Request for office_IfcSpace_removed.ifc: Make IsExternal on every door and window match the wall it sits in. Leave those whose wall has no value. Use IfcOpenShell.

First a look at what the model holds.

```python
import ifcopenshell
import ifcopenshell.util.element

model = ifcopenshell.open("office_IfcSpace_removed.ifc")
print(model.schema)
seen = {}
for e in model.by_type("IfcDoor") + model.by_type("IfcWindow"):
    if not e.FillsVoids:
        continue
    host = e.FillsVoids[0].RelatingOpeningElement.VoidsElements[0].RelatingBuildingElement
    own = ifcopenshell.util.element.get_pset(e, f"Pset_{e.is_a()[3:].removesuffix('StandardCase')}Common", "IsExternal")
    wall = ifcopenshell.util.element.get_pset(host, "Pset_WallCommon", "IsExternal")
    seen[e.is_a(), own, wall] = seen.get((e.is_a(), own, wall), 0) + 1
for (cls, own, wall), count in sorted(seen.items(), key=str):
    print(count, cls, "IsExternal:", own, "| host wall:", wall)
```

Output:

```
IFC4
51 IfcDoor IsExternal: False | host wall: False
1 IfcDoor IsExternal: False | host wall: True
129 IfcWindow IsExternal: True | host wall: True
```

```python
import ifcopenshell
import ifcopenshell.api.pset
import ifcopenshell.util.element

model = ifcopenshell.open("office_IfcSpace_removed.ifc")

count = 0
for ifc_class, pset_name in (("IfcDoor", "Pset_DoorCommon"), ("IfcWindow", "Pset_WindowCommon")):
    for e in model.by_type(ifc_class):
        if not e.FillsVoids:
            continue
        host = e.FillsVoids[0].RelatingOpeningElement.VoidsElements[0].RelatingBuildingElement
        external = ifcopenshell.util.element.get_pset(host, "Pset_WallCommon", "IsExternal")
        if external is None or ifcopenshell.util.element.get_pset(e, pset_name, "IsExternal") == external:
            continue
        pset = ifcopenshell.api.pset.add_pset(model, product=e, name=pset_name)
        ifcopenshell.api.pset.edit_pset(model, pset=pset, properties={"IsExternal": external})
        count += 1

print(count, "updated")

model.write("office_IfcSpace_removed_updated.ifc")
```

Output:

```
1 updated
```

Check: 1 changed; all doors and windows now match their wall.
